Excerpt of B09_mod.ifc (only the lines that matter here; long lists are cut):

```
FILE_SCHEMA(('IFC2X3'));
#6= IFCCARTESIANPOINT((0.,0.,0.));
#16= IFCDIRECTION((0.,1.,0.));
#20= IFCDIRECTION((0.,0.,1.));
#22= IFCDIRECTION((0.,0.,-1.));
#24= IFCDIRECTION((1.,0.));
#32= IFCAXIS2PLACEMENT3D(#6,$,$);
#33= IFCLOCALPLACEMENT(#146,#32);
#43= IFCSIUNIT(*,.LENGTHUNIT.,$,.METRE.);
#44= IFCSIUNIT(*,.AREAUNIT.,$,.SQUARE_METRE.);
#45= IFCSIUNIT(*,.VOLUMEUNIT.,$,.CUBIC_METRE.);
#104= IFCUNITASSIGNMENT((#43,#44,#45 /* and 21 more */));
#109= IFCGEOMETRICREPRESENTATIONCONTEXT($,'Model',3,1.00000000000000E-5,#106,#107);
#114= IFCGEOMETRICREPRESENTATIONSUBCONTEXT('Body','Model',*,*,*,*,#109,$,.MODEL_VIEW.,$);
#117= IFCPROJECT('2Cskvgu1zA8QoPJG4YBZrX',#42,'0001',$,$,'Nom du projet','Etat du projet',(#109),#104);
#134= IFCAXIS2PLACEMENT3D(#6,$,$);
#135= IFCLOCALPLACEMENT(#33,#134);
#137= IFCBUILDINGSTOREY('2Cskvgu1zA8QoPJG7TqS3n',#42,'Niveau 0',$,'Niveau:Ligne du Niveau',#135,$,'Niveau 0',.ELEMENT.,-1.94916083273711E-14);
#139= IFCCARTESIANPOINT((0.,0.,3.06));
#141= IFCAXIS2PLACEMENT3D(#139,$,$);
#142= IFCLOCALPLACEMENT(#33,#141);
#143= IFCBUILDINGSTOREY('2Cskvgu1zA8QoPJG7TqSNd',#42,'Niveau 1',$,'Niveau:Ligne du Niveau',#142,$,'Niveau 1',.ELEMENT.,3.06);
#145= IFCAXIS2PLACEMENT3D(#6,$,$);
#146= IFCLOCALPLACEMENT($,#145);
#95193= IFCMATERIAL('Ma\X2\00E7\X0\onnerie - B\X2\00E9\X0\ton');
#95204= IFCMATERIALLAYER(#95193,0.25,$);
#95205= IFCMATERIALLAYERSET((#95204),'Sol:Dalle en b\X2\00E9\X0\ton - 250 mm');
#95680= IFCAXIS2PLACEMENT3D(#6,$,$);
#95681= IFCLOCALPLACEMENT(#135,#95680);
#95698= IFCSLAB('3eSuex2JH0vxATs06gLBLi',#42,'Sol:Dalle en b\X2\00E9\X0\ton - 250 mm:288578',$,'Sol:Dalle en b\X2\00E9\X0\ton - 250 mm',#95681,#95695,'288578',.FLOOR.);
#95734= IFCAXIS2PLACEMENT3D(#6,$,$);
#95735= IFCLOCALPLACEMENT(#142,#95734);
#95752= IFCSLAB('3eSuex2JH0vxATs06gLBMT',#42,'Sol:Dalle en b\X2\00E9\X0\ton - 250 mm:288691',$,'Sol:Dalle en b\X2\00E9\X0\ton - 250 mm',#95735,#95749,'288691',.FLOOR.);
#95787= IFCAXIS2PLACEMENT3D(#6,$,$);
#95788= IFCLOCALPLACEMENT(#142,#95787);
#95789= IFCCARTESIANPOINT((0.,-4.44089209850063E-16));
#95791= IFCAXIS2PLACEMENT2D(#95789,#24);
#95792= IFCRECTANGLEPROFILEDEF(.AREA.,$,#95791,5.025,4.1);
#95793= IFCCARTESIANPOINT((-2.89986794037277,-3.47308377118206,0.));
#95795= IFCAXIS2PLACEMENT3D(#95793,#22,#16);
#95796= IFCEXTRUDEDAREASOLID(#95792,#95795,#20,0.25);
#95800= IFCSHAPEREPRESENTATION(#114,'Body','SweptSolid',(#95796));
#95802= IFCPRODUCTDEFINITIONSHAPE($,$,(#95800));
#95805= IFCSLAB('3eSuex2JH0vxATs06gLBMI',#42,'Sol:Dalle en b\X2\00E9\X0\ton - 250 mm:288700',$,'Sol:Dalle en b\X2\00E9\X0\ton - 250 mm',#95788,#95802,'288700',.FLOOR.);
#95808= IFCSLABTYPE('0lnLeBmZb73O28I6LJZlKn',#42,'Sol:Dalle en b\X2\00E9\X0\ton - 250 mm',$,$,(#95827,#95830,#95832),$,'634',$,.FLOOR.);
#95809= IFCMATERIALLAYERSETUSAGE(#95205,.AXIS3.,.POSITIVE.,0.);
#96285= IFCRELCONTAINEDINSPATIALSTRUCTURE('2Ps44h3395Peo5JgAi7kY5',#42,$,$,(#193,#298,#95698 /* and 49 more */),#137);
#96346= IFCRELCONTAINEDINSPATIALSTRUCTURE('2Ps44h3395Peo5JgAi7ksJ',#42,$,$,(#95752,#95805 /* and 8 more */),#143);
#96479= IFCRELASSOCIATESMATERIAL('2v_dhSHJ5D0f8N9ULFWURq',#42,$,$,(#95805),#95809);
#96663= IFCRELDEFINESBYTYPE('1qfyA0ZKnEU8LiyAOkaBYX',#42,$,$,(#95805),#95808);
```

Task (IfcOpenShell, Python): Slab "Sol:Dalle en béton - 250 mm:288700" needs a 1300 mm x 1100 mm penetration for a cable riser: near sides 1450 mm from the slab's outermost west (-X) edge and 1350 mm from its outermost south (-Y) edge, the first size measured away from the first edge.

```python
import numpy as np
import ifcopenshell
import ifcopenshell.api.feature
import ifcopenshell.api.geometry
import ifcopenshell.api.root
import ifcopenshell.geom
import ifcopenshell.util.placement
import ifcopenshell.util.representation
import ifcopenshell.util.shape
import ifcopenshell.util.unit

model = ifcopenshell.open("B09_mod.ifc")
unit_scale = ifcopenshell.util.unit.calculate_unit_scale(model)
settings = ifcopenshell.geom.settings()


def volume(element):
    """Net volume in cubic metres, openings subtracted."""
    shape = ifcopenshell.geom.create_shape(settings, element)
    return ifcopenshell.util.shape.get_volume(shape.geometry)


slab = model.by_id(95805)
before = volume(slab)

# Extent in the slab's own axes, in metres. The edges named are its -X and -Y sides.
slab_shape = ifcopenshell.geom.create_shape(settings, slab)
vertices = ifcopenshell.util.shape.get_vertices(slab_shape.geometry)
x_min, y_min, bottom = vertices.min(axis=0)
top = vertices[:, 2].max()

opening = ifcopenshell.api.root.create_entity(model, ifc_class="IfcOpeningElement", name="Cable riser opening")
context = ifcopenshell.util.representation.get_context(model, "Model", "Body", "MODEL_VIEW")
width, depth = 1.3, 1.1
outline = [(0.0, 0.0), (width, 0.0), (width, depth), (0.0, depth), (0.0, 0.0)]
# Overshoot both faces by 50 mm so the cut is clean.
shape = ifcopenshell.api.geometry.add_slab_representation(
    model, context=context, depth=top - bottom + 0.1, polyline=outline
)
ifcopenshell.api.geometry.assign_representation(model, product=opening, representation=shape)

matrix = ifcopenshell.util.placement.get_local_placement(slab.ObjectPlacement)
matrix[:, 3] = matrix @ np.append(np.array([x_min + 1.45, y_min + 1.35, bottom - 0.05]) / unit_scale, 1.0)
ifcopenshell.api.geometry.edit_object_placement(model, product=opening, matrix=matrix, is_si=False)
ifcopenshell.api.feature.add_feature(model, feature=opening, element=slab)

after = volume(slab)

print(f"slab volume {before:.3f} -> {after:.3f} m3")

model.write("B09_mod-out.ifc")
```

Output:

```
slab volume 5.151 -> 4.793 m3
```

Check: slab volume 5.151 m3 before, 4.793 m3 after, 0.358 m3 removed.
